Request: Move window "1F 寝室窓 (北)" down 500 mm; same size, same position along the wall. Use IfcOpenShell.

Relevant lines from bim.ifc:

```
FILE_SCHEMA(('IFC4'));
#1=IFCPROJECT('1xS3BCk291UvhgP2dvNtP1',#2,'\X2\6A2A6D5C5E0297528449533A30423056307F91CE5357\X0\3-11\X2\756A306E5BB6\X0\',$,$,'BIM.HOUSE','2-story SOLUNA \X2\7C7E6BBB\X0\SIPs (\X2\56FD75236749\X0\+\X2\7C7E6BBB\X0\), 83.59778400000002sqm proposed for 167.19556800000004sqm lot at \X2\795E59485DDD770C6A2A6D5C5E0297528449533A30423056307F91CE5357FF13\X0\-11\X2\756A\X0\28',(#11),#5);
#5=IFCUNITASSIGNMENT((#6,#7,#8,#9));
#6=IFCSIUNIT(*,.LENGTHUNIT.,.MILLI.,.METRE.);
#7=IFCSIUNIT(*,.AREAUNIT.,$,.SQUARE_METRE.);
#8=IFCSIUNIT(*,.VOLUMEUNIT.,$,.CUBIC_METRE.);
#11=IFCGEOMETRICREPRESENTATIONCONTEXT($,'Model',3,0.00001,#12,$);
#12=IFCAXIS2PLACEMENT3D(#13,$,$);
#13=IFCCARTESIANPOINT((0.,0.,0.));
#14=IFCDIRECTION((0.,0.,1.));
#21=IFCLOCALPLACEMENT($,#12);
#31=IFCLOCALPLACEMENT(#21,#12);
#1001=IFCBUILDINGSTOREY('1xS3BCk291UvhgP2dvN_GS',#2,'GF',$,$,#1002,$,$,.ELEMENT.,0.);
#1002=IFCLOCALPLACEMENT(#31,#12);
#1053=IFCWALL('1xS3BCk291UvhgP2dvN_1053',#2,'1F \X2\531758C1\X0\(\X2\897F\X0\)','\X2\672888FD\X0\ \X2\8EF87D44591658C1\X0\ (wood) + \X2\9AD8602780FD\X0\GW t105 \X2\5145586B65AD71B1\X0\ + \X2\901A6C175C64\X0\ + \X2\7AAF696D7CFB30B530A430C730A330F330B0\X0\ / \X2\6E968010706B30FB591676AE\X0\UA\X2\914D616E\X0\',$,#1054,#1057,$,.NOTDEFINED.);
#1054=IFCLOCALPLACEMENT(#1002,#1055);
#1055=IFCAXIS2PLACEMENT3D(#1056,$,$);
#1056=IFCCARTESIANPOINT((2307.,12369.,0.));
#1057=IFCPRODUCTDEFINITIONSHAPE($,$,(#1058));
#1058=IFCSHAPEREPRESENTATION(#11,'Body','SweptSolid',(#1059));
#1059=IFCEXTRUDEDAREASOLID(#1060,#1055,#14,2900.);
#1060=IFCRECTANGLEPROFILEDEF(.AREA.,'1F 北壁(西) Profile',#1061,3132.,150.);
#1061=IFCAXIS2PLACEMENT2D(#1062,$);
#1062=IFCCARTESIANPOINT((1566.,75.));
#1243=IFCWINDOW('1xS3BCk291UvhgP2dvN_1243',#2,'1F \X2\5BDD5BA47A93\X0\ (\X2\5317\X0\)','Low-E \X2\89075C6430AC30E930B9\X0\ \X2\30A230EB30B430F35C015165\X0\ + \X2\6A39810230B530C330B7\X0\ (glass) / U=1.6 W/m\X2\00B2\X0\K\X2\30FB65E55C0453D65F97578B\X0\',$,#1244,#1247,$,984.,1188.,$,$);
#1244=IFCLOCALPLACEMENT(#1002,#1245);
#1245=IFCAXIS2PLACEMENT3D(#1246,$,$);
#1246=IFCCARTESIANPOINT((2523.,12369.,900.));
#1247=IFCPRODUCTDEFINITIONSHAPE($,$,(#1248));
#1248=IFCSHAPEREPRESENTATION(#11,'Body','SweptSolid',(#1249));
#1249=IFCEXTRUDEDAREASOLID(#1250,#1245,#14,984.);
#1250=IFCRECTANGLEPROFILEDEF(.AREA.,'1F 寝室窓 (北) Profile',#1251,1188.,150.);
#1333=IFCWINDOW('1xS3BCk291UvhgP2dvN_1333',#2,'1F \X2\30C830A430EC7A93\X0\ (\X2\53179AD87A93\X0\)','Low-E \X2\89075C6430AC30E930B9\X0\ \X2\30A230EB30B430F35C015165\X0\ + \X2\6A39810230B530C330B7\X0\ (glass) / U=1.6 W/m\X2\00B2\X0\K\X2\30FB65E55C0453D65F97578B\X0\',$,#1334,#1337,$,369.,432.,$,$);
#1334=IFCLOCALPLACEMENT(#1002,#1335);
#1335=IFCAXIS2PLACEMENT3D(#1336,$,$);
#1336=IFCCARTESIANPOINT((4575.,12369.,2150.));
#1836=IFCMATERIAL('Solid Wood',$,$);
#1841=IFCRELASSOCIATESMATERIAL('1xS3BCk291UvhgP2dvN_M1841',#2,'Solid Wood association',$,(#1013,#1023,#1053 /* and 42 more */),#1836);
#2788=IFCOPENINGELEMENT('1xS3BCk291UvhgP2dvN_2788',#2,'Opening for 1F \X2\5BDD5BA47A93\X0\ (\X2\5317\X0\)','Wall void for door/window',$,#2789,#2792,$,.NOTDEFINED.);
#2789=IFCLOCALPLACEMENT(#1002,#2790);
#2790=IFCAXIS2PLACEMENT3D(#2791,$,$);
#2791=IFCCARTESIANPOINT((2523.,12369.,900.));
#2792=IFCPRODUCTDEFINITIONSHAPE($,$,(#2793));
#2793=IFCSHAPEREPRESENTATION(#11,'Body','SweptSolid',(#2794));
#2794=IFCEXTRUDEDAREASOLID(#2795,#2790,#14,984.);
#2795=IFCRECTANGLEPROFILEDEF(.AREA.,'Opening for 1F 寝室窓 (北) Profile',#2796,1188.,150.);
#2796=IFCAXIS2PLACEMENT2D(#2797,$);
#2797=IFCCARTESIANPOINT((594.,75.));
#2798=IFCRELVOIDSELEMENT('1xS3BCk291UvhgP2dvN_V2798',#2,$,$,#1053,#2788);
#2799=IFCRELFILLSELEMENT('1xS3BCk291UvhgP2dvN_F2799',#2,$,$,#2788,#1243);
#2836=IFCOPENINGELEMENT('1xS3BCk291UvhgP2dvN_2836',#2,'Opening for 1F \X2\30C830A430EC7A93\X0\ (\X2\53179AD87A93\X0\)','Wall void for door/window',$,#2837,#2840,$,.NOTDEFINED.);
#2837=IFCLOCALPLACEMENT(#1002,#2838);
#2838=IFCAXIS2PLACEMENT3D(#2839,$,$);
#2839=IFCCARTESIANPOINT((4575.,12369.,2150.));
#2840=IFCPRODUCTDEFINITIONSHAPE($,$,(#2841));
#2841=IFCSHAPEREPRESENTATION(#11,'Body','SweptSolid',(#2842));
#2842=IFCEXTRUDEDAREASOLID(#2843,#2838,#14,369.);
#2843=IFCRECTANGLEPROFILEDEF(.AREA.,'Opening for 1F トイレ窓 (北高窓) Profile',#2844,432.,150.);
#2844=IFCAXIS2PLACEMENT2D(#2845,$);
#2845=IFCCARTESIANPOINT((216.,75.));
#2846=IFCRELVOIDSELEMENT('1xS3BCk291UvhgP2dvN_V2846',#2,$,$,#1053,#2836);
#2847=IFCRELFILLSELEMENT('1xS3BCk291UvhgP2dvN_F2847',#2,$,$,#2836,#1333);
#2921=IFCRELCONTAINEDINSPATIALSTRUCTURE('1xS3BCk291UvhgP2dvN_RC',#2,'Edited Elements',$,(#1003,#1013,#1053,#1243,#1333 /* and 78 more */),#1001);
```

```python
import numpy as np
import ifcopenshell
import ifcopenshell.api.geometry
import ifcopenshell.util.placement
import ifcopenshell.util.unit

model = ifcopenshell.open("bim.ifc")
unit_scale = ifcopenshell.util.unit.calculate_unit_scale(model)

window = model.by_guid("1xS3BCk291UvhgP2dvN_1243")
opening = window.FillsVoids[0].RelatingOpeningElement
dz = -0.5 / unit_scale

shift = np.array([0.0, 0.0, dz])
# The window is not placed relative to its opening, so move both.
for product in (opening, window):
    matrix = ifcopenshell.util.placement.get_local_placement(product.ObjectPlacement)
    matrix[:3, 3] += shift
    ifcopenshell.api.geometry.edit_object_placement(model, product=product, matrix=matrix, is_si=False)

print(f"moved by {dz * unit_scale:+.3f} m")

model.write("bim-out.ifc")
```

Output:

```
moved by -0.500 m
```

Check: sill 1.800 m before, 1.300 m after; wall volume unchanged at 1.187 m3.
